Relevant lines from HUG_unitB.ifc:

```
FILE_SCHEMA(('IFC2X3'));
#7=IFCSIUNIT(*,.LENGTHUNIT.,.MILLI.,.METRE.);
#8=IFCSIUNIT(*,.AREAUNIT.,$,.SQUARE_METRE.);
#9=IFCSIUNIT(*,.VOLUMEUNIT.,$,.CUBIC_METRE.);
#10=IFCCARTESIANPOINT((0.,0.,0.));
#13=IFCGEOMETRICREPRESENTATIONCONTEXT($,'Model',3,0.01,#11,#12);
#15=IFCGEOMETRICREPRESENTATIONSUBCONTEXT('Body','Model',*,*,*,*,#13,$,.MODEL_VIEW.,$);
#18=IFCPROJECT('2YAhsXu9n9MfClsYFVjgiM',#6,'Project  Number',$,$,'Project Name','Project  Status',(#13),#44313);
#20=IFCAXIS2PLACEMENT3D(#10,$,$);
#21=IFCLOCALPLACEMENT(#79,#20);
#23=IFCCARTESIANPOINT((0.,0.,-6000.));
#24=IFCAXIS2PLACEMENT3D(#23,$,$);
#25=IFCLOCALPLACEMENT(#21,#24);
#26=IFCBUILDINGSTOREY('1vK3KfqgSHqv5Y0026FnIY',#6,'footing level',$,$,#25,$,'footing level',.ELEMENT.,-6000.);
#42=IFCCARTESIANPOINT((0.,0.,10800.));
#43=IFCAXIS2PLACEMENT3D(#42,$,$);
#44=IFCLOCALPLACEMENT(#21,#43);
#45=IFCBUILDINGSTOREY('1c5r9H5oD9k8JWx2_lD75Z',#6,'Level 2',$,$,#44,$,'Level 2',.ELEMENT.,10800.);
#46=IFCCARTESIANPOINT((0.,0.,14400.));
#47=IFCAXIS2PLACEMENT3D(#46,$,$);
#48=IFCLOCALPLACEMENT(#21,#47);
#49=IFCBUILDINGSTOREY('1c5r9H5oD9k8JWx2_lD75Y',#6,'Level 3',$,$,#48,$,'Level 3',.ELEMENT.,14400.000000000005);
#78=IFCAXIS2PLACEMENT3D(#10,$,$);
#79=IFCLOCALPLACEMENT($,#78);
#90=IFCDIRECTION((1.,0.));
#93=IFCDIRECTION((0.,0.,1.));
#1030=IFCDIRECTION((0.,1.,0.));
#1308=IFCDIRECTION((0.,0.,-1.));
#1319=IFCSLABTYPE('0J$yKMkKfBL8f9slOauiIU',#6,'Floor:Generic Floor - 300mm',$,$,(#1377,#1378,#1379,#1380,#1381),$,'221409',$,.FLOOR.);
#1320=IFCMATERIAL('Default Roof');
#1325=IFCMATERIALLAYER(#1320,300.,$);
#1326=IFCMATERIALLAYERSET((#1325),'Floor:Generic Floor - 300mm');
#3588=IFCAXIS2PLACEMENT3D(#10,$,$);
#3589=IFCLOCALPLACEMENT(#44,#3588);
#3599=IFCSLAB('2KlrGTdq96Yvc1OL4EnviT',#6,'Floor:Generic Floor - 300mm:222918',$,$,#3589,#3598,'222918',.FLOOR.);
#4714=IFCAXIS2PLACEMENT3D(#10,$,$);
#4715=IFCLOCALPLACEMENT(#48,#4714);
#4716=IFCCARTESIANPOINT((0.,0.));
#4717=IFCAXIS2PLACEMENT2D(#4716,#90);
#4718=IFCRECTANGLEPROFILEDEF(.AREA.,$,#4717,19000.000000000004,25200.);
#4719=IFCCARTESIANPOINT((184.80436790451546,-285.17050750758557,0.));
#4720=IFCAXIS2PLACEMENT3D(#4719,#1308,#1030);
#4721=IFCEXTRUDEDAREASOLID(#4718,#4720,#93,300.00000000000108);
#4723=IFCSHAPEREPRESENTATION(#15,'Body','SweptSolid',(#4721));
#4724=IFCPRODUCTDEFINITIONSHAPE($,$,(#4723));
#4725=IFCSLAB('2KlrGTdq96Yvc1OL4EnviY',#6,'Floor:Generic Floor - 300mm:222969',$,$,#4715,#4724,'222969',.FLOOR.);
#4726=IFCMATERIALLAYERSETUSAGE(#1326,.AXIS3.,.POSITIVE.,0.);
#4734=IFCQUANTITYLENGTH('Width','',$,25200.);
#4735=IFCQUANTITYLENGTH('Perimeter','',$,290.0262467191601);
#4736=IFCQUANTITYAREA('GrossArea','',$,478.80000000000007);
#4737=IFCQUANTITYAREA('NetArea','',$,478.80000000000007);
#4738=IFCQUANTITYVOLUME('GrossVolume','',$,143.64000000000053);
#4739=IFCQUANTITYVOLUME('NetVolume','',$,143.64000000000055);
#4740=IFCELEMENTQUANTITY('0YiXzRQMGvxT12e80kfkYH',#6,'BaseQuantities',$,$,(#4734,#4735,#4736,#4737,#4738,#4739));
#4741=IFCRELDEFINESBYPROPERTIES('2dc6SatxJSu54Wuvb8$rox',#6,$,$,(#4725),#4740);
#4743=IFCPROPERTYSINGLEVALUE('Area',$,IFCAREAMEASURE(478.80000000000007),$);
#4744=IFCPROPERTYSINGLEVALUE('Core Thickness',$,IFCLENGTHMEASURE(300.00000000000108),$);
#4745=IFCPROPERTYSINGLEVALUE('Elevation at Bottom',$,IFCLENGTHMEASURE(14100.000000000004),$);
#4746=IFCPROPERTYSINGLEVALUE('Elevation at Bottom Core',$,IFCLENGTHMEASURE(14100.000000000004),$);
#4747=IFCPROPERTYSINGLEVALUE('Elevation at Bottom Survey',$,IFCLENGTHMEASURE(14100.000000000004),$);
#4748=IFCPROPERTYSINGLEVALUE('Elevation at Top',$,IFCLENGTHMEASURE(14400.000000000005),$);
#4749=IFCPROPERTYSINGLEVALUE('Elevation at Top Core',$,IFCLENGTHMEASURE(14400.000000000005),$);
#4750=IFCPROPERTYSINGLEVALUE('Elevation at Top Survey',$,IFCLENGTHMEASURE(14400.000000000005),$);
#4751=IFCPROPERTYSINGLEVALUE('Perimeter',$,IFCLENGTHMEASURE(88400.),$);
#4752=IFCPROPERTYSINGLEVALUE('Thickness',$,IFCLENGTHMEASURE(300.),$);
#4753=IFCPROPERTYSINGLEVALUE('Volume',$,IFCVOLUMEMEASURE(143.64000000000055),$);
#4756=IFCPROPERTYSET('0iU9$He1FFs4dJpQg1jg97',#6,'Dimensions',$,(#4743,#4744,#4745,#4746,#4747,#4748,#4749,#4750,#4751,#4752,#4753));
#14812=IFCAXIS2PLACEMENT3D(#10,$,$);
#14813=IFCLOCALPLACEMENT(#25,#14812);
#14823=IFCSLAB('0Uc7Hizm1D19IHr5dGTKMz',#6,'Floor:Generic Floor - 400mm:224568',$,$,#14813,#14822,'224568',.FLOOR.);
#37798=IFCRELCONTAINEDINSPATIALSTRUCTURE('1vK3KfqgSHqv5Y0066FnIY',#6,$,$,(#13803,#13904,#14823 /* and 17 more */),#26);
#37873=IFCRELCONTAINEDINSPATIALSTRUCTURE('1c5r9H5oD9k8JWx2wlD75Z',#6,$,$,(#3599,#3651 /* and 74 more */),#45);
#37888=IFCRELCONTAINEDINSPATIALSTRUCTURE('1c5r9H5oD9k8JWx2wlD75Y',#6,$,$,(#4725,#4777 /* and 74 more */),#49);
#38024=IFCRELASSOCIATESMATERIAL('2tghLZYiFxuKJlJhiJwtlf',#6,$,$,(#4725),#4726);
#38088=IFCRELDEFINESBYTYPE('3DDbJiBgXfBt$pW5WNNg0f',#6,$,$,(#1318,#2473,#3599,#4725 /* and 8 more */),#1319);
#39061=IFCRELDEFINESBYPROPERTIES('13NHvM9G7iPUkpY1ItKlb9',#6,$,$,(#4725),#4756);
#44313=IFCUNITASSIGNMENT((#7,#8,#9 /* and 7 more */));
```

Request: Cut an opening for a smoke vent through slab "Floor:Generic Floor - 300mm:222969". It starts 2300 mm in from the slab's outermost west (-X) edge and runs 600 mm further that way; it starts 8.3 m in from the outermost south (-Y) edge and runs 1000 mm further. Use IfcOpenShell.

```python
import numpy as np
import ifcopenshell
import ifcopenshell.api.feature
import ifcopenshell.api.geometry
import ifcopenshell.api.pset
import ifcopenshell.api.root
import ifcopenshell.geom
import ifcopenshell.util.element
import ifcopenshell.util.placement
import ifcopenshell.util.representation
import ifcopenshell.util.shape
import ifcopenshell.util.unit

model = ifcopenshell.open("HUG_unitB.ifc")
unit_scale = ifcopenshell.util.unit.calculate_unit_scale(model)
area_scale = ifcopenshell.util.unit.calculate_unit_scale(model, "AREAUNIT")
volume_scale = ifcopenshell.util.unit.calculate_unit_scale(model, "VOLUMEUNIT")
settings = ifcopenshell.geom.settings()


def volume(element):
    """Net volume in cubic metres, openings subtracted."""
    shape = ifcopenshell.geom.create_shape(settings, element)
    return ifcopenshell.util.shape.get_volume(shape.geometry)


slab = model.by_guid("2KlrGTdq96Yvc1OL4EnviY")
before = volume(slab)

# Extent in the slab's own axes, in metres. The edges named are its -X and -Y sides.
slab_shape = ifcopenshell.geom.create_shape(settings, slab)
vertices = ifcopenshell.util.shape.get_vertices(slab_shape.geometry)
x_min, y_min, bottom = vertices.min(axis=0)
top = vertices[:, 2].max()

opening = ifcopenshell.api.root.create_entity(model, ifc_class="IfcOpeningElement", name="Smoke vent opening")
context = ifcopenshell.util.representation.get_context(model, "Model", "Body", "MODEL_VIEW")
width, depth = 0.6, 1
outline = [(0.0, 0.0), (width, 0.0), (width, depth), (0.0, depth), (0.0, 0.0)]
# Overshoot both faces by 50 mm so the cut is clean.
shape = ifcopenshell.api.geometry.add_slab_representation(
    model, context=context, depth=top - bottom + 0.1, polyline=outline
)
ifcopenshell.api.geometry.assign_representation(model, product=opening, representation=shape)

matrix = ifcopenshell.util.placement.get_local_placement(slab.ObjectPlacement)
matrix[:, 3] = matrix @ np.append(np.array([x_min + 2.3, y_min + 8.3, bottom - 0.05]) / unit_scale, 1.0)
ifcopenshell.api.geometry.edit_object_placement(model, product=opening, matrix=matrix, is_si=False)
ifcopenshell.api.feature.add_feature(model, feature=opening, element=slab)

after = volume(slab)

# Update the slab's stored quantities.
qto = model.by_id(ifcopenshell.util.element.get_pset(slab, "BaseQuantities", should_inherit=False)["id"])
ifcopenshell.api.pset.edit_qto(model, qto=qto, properties={
    "NetArea": after / (top - bottom) / area_scale,
    "NetVolume": after / volume_scale,
})
pset = model.by_id(ifcopenshell.util.element.get_pset(slab, "Dimensions", should_inherit=False)["id"])
ifcopenshell.api.pset.edit_pset(model, pset=pset, properties={
    "Area": model.create_entity("IfcAreaMeasure", after / (top - bottom) / area_scale),
    "Volume": model.create_entity("IfcVolumeMeasure", after / volume_scale),
})

print(f"slab volume {before:.3f} -> {after:.3f} m3")

model.write("HUG_unitB_rev.ifc")
```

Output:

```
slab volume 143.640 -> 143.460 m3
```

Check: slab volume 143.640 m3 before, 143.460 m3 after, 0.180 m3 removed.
